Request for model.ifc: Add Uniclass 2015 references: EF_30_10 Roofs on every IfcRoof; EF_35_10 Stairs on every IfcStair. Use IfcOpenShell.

First a look at what the model holds.

```python
import ifcopenshell

model = ifcopenshell.open("model.ifc")
print(model.schema)
print("classifications:", [c.Name for c in model.by_type("IfcClassification")])
for ifc_class in ("IfcDoor", "IfcRoof", "IfcStair", "IfcWall", "IfcWindow"):
    print(ifc_class, len(model.by_type(ifc_class)))
```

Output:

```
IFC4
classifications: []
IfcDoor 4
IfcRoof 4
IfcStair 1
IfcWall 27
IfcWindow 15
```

```python
import ifcopenshell
import ifcopenshell.api.classification

model = ifcopenshell.open("model.ifc")

system = ifcopenshell.api.classification.add_classification(model, classification="Uniclass 2015")

codes = {
    "IfcRoof": ("EF_30_10", "Roofs"),
    "IfcStair": ("EF_35_10", "Stairs"),
}
for ifc_class, (code, name) in codes.items():
    products = model.by_type(ifc_class)
    ifcopenshell.api.classification.add_reference(
        model, products=products, classification=system, identification=code, name=name
    )
    print(code, len(products))

model.write("model_rev.ifc")
```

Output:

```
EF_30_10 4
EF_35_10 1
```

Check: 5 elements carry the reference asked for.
